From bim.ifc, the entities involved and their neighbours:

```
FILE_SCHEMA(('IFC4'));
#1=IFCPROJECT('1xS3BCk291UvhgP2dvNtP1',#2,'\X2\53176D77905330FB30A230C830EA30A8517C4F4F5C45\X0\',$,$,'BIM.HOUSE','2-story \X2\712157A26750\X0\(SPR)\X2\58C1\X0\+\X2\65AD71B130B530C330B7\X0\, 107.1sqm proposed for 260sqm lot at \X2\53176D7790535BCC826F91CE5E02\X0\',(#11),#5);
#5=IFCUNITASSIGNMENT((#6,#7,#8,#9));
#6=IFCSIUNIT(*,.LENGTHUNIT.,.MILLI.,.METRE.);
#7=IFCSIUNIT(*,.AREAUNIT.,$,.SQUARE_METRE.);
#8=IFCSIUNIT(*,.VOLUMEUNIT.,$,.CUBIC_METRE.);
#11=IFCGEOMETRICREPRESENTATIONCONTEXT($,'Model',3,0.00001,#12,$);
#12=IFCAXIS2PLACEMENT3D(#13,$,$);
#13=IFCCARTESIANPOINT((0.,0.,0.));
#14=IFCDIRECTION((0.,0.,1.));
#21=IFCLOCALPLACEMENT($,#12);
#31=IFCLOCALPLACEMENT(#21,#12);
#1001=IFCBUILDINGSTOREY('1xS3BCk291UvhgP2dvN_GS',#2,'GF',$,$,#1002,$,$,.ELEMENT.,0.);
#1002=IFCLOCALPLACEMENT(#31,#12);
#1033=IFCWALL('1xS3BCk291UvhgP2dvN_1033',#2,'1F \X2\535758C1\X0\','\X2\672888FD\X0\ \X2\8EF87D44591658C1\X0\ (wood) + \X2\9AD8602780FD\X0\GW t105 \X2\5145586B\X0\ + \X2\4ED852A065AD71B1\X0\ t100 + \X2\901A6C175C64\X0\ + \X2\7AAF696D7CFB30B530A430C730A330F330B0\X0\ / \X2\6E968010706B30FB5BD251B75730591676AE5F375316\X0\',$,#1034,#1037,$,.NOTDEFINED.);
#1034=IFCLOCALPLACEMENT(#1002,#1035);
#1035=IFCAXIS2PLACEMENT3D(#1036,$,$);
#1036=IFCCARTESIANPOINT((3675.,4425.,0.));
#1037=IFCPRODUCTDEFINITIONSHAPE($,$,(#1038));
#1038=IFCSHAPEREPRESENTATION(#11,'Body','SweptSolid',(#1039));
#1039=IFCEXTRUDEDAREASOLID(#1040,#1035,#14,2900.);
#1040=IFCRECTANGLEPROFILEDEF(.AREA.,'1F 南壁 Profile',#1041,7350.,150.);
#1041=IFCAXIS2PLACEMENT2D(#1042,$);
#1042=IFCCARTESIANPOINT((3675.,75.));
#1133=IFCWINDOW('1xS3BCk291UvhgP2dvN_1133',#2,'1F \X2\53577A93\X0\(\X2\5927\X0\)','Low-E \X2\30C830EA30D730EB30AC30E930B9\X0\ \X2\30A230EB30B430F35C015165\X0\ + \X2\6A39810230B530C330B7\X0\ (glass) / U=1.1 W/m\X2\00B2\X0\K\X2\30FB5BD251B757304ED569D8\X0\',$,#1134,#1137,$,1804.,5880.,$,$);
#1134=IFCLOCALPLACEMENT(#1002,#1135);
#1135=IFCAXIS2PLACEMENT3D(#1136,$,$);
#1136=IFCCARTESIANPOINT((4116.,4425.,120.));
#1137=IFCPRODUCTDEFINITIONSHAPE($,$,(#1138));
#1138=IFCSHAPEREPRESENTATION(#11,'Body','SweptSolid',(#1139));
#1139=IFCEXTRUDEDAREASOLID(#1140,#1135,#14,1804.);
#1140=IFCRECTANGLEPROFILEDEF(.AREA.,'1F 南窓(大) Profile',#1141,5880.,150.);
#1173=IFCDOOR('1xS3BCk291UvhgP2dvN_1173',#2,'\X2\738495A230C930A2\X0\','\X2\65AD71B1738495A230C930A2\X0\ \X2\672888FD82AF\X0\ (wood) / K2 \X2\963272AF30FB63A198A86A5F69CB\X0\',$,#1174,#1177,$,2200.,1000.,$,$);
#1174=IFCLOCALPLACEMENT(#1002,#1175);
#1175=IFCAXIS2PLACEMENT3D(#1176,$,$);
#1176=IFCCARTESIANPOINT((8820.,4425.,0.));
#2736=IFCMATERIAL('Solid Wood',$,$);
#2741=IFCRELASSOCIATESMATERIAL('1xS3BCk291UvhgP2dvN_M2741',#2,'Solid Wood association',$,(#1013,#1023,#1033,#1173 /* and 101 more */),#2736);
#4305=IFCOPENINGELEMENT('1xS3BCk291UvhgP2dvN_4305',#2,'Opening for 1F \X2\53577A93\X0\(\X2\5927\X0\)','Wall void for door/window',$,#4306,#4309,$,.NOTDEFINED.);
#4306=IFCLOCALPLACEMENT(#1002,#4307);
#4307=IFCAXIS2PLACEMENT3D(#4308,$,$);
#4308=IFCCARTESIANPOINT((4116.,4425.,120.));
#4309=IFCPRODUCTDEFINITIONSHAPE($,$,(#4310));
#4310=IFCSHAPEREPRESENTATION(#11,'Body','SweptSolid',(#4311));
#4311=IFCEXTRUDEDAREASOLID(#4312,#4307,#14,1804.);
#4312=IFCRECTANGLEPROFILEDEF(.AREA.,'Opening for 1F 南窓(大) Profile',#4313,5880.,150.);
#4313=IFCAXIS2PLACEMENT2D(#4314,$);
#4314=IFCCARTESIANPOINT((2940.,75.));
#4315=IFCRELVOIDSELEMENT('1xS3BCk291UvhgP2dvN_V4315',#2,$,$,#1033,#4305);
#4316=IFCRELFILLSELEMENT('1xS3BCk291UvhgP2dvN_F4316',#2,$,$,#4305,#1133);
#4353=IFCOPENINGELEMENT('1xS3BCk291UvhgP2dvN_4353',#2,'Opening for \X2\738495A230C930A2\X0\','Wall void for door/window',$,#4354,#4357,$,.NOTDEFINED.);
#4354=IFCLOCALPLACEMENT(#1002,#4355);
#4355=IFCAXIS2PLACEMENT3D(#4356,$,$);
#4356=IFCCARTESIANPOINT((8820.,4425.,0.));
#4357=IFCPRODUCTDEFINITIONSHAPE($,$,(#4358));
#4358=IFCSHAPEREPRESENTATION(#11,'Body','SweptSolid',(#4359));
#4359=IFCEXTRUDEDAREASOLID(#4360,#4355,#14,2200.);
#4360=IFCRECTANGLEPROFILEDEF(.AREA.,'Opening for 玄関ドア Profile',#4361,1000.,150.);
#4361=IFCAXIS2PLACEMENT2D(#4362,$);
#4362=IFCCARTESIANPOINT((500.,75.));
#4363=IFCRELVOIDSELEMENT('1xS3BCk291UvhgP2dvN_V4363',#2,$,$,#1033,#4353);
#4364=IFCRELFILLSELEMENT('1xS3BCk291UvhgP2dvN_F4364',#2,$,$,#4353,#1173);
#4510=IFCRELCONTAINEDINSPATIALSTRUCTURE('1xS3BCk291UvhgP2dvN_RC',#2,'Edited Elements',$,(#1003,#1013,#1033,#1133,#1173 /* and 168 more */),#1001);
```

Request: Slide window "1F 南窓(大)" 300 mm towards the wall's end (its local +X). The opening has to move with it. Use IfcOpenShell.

```python
import ifcopenshell
import ifcopenshell.api.geometry
import ifcopenshell.util.placement

model = ifcopenshell.open("bim.ifc")

window = model.by_guid("1xS3BCk291UvhgP2dvN_1133")
opening = window.FillsVoids[0].RelatingOpeningElement
wall = opening.VoidsElements[0].RelatingBuildingElement

wall_matrix = ifcopenshell.util.placement.get_local_placement(wall.ObjectPlacement)
shift = wall_matrix[:3, 0] * 300.0
before = ifcopenshell.util.placement.get_local_placement(window.ObjectPlacement)[:3, 3].copy()

# The window is not placed relative to its opening, so move both.
for product in (opening, window):
    matrix = ifcopenshell.util.placement.get_local_placement(product.ObjectPlacement)
    matrix[:3, 3] += shift
    ifcopenshell.api.geometry.edit_object_placement(model, product=product, matrix=matrix, is_si=False)

after = ifcopenshell.util.placement.get_local_placement(window.ObjectPlacement)[:3, 3]
print("window moved by", (after - before).round(3) + 0.0)

model.write("bim-out.ifc")
```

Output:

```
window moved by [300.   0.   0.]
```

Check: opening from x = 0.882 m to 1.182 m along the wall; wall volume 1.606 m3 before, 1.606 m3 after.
